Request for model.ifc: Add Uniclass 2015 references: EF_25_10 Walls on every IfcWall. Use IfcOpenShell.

First a look at what the model holds.

```python
import ifcopenshell

model = ifcopenshell.open("model.ifc")
print(model.schema)
print("classifications:", [c.Name for c in model.by_type("IfcClassification")])
for ifc_class in ("IfcDoor", "IfcRoof", "IfcStair", "IfcWall", "IfcWindow"):
    print(ifc_class, len(model.by_type(ifc_class)))
```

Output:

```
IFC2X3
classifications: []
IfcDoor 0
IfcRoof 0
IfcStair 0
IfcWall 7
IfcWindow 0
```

```python
import ifcopenshell
import ifcopenshell.api.classification

model = ifcopenshell.open("model.ifc")

# IFC2X3 requires Source and Edition and has no link from the project to the system.
system = model.create_entity("IfcClassification", Source="NBS", Edition="2015", Name="Uniclass 2015")

codes = {
    "IfcWall": ("EF_25_10", "Walls"),
}
for ifc_class, (code, name) in codes.items():
    products = model.by_type(ifc_class)
    ifcopenshell.api.classification.add_reference(
        model, products=products, classification=system, identification=code, name=name
    )
    print(code, len(products))

model.write("model_rev.ifc")
```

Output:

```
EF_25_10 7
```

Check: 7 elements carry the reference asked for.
